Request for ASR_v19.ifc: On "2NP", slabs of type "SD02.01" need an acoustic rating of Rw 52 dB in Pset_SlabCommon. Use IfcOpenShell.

First a look at what the model holds.

```python
import ifcopenshell
import ifcopenshell.util.element

model = ifcopenshell.open("ASR_v19.ifc")
print(model.schema)
storey = next(s for s in model.by_type("IfcBuildingStorey") if s.Name == "2NP")
slabs = [e for e in ifcopenshell.util.element.get_decomposition(storey) if e.is_a("IfcSlab")]
seen = {}
for e in slabs:
    element_type = ifcopenshell.util.element.get_type(e)
    key = (element_type.Name if element_type != e and element_type else None, ifcopenshell.util.element.get_pset(e, "Pset_SlabCommon", "AcousticRating"))
    seen[key] = seen.get(key, 0) + 1
for (name, value), count in sorted(seen.items(), key=str):
    print(count, "x", name, "|", value)
```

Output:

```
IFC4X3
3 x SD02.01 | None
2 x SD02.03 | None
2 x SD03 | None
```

```python
import ifcopenshell
import ifcopenshell.api.pset
import ifcopenshell.util.element

model = ifcopenshell.open("ASR_v19.ifc")

storey = next(s for s in model.by_type("IfcBuildingStorey") if s.Name == "2NP")
slabs = [e for e in ifcopenshell.util.element.get_decomposition(storey) if e.is_a("IfcSlab")]

count = 0
for e in slabs:
    element_type = ifcopenshell.util.element.get_type(e)
    if element_type in (None, e) or element_type.Name != "SD02.01":
        continue
    # add_pset returns the element's existing set when there is one.
    pset = ifcopenshell.api.pset.add_pset(model, product=e, name="Pset_SlabCommon")
    ifcopenshell.api.pset.edit_pset(model, pset=pset, properties={"AcousticRating": "Rw 52 dB"})
    count += 1

print(count, "slabs updated")

model.write("ASR_v19_v2.ifc")
```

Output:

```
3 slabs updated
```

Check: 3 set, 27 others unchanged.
